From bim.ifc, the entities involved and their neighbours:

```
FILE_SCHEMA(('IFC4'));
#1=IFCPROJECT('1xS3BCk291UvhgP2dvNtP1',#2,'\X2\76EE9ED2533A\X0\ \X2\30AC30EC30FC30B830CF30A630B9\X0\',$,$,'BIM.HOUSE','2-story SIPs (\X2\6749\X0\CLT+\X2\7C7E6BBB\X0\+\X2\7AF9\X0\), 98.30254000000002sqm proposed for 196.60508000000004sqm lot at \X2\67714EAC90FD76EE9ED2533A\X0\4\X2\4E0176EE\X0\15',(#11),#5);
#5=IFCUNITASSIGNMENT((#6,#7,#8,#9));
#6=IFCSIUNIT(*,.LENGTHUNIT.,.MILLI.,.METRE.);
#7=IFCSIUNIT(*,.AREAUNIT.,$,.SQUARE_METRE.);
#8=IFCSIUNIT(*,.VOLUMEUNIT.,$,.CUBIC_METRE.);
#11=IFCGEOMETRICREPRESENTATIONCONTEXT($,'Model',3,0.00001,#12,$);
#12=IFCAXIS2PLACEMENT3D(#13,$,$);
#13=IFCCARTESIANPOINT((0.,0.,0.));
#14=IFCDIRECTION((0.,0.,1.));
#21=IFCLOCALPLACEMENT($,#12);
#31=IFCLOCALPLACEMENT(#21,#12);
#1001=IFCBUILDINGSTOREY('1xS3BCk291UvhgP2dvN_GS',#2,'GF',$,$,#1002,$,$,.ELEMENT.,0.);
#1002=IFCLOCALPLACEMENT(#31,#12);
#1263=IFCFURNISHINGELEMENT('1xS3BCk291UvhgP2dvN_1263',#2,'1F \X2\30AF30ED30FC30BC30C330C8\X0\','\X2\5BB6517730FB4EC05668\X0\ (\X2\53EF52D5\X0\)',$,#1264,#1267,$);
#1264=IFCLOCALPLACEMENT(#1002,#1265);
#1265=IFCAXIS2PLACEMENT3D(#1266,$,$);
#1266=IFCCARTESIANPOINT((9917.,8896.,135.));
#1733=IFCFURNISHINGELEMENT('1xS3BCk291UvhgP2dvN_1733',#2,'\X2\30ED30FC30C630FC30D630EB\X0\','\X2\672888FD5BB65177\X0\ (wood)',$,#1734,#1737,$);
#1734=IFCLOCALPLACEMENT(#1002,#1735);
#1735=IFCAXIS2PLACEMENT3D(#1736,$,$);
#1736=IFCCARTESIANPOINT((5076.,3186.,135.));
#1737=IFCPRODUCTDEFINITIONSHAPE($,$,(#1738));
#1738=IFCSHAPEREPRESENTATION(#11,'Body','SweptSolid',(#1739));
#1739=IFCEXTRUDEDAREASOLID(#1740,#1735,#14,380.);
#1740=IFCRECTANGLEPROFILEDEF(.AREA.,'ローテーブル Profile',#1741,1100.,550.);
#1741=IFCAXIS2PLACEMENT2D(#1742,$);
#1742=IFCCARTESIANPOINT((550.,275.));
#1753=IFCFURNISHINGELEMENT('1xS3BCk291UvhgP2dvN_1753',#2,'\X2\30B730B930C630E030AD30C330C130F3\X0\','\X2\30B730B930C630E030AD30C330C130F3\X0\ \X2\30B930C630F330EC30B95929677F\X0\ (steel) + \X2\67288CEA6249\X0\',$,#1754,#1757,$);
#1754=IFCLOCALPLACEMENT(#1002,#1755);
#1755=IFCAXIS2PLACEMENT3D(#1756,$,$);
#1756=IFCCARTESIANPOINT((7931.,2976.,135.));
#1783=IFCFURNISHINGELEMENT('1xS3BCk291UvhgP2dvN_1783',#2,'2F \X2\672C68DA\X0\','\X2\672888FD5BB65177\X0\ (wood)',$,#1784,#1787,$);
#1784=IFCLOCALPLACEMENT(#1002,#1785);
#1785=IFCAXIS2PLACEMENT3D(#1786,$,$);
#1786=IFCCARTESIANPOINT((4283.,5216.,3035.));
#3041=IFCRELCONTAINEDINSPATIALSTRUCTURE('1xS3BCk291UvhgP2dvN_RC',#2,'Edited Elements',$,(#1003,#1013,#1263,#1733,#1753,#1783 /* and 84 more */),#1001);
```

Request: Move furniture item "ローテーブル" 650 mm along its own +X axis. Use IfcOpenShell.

```python
import ifcopenshell
import ifcopenshell.api.geometry
import ifcopenshell.util.placement
import ifcopenshell.util.unit

model = ifcopenshell.open("bim.ifc")
unit_scale = ifcopenshell.util.unit.calculate_unit_scale(model)

item = model.by_id(1733)
matrix = ifcopenshell.util.placement.get_local_placement(item.ObjectPlacement)
matrix[:3, 3] += matrix[:3, 0] * 0.65 / unit_scale
ifcopenshell.api.geometry.edit_object_placement(model, product=item, matrix=matrix, is_si=False)

print(ifcopenshell.util.placement.get_local_placement(item.ObjectPlacement).round(3) + 0.0)

model.write("bim_rev.ifc")
```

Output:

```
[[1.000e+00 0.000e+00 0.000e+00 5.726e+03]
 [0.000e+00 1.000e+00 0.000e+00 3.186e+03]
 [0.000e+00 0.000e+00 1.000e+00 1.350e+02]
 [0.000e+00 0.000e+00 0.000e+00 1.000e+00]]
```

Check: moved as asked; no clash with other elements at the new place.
